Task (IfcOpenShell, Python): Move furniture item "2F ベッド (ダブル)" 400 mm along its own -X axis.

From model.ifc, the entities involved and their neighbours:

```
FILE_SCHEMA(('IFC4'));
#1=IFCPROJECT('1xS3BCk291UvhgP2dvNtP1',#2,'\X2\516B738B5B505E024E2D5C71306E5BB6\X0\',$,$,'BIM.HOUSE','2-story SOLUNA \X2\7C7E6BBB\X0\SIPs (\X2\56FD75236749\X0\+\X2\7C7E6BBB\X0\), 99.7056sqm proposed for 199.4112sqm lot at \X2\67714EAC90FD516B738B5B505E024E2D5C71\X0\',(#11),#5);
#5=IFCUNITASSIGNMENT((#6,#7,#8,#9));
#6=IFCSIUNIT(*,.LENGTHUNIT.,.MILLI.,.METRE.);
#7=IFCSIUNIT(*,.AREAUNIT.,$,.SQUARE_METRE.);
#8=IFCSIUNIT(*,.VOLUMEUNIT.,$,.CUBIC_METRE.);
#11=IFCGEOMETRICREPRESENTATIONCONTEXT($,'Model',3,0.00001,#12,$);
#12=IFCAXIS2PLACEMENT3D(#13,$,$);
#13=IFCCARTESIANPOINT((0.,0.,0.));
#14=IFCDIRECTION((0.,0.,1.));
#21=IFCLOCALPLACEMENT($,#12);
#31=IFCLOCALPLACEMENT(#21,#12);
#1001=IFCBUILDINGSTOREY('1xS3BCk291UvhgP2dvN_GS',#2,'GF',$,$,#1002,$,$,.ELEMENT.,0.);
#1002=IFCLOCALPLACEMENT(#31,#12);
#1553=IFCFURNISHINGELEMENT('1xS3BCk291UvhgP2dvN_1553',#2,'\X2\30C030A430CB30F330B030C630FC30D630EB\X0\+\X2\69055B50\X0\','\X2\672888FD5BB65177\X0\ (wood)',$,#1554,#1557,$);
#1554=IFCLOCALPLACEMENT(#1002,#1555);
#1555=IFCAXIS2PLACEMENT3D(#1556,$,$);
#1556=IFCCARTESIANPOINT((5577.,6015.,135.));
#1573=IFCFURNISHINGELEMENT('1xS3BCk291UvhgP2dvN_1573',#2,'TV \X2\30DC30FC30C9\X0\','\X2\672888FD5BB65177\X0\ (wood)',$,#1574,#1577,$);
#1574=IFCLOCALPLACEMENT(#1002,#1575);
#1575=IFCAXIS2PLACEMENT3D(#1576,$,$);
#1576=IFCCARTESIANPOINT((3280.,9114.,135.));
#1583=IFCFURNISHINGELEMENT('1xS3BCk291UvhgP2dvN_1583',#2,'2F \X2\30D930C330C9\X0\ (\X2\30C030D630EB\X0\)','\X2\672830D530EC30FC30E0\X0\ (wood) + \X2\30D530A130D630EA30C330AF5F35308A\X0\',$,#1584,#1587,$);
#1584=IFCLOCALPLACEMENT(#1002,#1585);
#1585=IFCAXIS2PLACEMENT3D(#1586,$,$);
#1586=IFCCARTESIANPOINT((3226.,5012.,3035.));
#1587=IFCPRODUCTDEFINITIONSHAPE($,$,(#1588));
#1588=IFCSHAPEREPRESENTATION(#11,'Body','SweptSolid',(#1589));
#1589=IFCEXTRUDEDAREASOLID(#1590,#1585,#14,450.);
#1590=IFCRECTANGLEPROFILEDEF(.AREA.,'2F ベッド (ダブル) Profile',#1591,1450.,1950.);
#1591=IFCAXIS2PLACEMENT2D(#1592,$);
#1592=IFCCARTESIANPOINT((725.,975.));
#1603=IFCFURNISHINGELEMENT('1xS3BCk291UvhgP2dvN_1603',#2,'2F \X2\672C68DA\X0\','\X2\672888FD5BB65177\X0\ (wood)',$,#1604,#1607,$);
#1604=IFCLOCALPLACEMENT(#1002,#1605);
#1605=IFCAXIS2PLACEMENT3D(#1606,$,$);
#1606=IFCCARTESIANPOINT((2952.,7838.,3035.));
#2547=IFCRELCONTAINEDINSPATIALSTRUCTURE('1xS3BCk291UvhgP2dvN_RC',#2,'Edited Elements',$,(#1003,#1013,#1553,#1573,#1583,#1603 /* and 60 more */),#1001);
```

```python
import ifcopenshell
import ifcopenshell.api.geometry
import ifcopenshell.util.placement
import ifcopenshell.util.unit

model = ifcopenshell.open("model.ifc")
unit_scale = ifcopenshell.util.unit.calculate_unit_scale(model)

item = model.by_guid("1xS3BCk291UvhgP2dvN_1583")
matrix = ifcopenshell.util.placement.get_local_placement(item.ObjectPlacement)
matrix[:3, 3] -= matrix[:3, 0] * 0.4 / unit_scale
ifcopenshell.api.geometry.edit_object_placement(model, product=item, matrix=matrix, is_si=False)

print(ifcopenshell.util.placement.get_local_placement(item.ObjectPlacement).round(3) + 0.0)

model.write("model-out.ifc")
```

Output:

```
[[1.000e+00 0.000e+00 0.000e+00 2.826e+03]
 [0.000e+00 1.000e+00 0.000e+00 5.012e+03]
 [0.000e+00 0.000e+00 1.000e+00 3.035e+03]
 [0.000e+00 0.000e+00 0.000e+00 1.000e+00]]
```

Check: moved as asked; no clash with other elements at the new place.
